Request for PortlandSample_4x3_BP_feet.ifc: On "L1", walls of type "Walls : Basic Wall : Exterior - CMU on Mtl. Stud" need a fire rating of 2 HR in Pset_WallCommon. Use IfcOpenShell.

First a look at what the model holds.

```python
import ifcopenshell
import ifcopenshell.util.element

model = ifcopenshell.open("PortlandSample_4x3_BP_feet.ifc")
print(model.schema)
storey = next(s for s in model.by_type("IfcBuildingStorey") if s.Name == "L1")
walls = [e for e in ifcopenshell.util.element.get_decomposition(storey) if e.is_a("IfcWall")]
seen = {}
for e in walls:
    element_type = ifcopenshell.util.element.get_type(e)
    key = (element_type.Name if element_type != e and element_type else None, ifcopenshell.util.element.get_pset(e, "Pset_WallCommon", "FireRating"))
    seen[key] = seen.get(key, 0) + 1
for (name, value), count in sorted(seen.items(), key=str):
    print(count, "x", name, "|", value)
```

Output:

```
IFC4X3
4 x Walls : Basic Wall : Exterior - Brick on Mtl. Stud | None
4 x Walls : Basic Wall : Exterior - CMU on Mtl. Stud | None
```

```python
import ifcopenshell
import ifcopenshell.api.pset
import ifcopenshell.util.element

model = ifcopenshell.open("PortlandSample_4x3_BP_feet.ifc")

storey = next(s for s in model.by_type("IfcBuildingStorey") if s.Name == "L1")
walls = [e for e in ifcopenshell.util.element.get_decomposition(storey) if e.is_a("IfcWall")]

count = 0
for e in walls:
    element_type = ifcopenshell.util.element.get_type(e)
    if element_type in (None, e) or element_type.Name != "Walls : Basic Wall : Exterior - CMU on Mtl. Stud":
        continue
    # add_pset returns the element's existing set when there is one.
    pset = ifcopenshell.api.pset.add_pset(model, product=e, name="Pset_WallCommon")
    ifcopenshell.api.pset.edit_pset(model, pset=pset, properties={"FireRating": "2 HR"})
    count += 1

print(count, "walls updated")

model.write("PortlandSample_4x3_BP_feet_rev.ifc")
```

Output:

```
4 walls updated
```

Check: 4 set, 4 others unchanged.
